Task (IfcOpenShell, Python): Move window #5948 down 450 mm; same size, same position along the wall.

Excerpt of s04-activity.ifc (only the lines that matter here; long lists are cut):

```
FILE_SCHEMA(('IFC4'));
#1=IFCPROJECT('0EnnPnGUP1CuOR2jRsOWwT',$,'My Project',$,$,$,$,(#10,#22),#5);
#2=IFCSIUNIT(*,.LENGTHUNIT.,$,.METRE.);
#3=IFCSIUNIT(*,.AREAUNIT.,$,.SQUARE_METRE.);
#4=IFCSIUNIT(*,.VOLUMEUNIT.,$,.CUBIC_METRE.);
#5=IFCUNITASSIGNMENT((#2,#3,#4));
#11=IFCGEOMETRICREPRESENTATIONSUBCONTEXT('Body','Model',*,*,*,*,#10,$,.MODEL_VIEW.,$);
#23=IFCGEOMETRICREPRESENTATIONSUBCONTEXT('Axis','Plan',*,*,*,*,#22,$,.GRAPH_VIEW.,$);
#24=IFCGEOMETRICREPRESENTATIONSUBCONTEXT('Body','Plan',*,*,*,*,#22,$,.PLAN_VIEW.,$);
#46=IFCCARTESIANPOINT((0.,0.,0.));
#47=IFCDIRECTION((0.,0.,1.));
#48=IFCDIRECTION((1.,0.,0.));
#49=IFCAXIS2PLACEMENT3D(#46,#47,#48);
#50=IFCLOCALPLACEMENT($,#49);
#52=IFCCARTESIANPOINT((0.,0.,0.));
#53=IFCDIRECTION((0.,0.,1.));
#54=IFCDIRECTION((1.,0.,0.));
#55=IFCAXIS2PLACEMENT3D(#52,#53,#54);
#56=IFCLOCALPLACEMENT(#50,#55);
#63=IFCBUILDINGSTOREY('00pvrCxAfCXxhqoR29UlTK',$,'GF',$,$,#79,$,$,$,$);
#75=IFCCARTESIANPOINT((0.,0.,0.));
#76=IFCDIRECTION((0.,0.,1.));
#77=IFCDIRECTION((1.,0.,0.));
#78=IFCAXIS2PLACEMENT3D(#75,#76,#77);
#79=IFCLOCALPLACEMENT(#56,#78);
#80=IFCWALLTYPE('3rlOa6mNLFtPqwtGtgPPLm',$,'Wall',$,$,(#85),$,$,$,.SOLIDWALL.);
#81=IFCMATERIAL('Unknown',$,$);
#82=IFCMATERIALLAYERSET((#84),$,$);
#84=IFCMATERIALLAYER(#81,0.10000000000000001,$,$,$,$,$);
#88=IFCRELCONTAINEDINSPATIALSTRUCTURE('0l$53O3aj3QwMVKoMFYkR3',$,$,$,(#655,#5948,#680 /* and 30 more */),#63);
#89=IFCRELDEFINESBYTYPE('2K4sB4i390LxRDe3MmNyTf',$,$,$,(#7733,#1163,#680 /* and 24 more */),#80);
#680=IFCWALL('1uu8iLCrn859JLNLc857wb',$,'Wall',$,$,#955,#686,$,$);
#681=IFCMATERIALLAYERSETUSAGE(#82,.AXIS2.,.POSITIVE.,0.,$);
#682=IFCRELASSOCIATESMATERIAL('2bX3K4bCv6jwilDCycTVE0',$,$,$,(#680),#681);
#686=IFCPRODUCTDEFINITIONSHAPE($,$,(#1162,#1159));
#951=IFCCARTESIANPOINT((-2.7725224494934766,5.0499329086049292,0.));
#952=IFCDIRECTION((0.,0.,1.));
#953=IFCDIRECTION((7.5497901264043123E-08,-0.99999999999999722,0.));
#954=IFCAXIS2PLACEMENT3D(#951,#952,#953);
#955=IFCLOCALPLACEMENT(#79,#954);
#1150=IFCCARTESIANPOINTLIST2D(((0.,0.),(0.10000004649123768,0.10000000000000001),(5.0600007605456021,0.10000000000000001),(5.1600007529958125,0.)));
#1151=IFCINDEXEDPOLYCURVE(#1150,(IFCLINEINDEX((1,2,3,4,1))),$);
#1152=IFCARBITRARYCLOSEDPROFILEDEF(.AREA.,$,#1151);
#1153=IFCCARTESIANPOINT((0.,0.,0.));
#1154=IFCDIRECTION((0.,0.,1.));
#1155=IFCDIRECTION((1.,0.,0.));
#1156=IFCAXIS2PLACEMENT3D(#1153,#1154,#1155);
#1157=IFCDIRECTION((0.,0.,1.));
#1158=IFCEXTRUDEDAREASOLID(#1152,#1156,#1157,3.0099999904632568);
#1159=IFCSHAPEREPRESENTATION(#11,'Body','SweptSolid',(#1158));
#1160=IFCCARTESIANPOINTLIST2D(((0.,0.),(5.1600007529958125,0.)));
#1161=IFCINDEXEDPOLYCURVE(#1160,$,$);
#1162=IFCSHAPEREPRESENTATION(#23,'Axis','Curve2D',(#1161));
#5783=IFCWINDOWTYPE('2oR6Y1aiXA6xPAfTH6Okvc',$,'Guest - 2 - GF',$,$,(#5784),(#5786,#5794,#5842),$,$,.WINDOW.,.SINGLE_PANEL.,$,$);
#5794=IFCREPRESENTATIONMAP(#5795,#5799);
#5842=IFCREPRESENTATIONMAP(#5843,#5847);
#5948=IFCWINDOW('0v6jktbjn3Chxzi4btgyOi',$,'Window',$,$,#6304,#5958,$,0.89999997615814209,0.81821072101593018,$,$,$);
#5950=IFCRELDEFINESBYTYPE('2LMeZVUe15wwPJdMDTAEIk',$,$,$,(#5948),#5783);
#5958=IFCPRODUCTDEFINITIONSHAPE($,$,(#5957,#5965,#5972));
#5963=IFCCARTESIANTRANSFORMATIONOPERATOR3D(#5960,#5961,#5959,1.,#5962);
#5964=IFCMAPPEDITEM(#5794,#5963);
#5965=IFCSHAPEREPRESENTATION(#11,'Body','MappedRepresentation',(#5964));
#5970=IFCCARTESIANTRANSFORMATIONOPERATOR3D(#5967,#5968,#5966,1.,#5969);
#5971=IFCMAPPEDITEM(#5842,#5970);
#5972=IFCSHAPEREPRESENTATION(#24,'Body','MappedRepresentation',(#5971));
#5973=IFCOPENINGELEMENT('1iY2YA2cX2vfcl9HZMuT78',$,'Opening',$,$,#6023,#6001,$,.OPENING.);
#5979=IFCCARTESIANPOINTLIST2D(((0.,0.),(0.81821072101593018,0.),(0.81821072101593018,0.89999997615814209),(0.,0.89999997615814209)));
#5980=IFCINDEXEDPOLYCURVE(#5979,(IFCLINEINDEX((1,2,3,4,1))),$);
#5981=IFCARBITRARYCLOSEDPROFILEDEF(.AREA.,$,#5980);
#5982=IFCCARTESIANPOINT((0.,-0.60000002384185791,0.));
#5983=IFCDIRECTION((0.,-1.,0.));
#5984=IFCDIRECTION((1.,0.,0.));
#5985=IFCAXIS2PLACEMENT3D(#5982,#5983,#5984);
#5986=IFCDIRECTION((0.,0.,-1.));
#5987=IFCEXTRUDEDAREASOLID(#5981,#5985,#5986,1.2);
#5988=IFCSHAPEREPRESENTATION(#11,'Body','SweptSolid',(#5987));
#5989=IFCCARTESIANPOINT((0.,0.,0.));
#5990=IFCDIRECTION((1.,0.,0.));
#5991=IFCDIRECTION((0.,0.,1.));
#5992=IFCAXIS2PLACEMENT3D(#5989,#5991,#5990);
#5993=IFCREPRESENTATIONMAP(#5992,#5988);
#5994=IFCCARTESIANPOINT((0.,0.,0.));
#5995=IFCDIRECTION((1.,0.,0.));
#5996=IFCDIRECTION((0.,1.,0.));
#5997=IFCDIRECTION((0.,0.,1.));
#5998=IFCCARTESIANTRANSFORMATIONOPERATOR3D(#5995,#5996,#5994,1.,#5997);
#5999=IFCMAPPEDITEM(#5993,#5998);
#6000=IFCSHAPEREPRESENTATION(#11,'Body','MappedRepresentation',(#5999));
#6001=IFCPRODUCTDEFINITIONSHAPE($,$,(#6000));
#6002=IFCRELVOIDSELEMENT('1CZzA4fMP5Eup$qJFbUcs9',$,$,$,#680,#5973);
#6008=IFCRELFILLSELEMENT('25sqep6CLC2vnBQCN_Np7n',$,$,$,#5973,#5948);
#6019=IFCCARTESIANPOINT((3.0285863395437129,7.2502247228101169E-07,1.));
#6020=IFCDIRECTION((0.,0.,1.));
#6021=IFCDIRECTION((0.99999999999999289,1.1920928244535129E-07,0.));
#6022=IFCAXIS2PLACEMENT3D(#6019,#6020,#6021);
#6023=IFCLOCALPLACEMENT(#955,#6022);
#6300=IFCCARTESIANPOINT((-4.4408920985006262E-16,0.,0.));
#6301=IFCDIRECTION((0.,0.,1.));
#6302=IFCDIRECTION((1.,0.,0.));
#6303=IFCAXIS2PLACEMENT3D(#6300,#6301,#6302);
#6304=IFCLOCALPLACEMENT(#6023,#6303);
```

```python
import numpy as np
import ifcopenshell
import ifcopenshell.api.geometry
import ifcopenshell.util.placement
import ifcopenshell.util.unit

model = ifcopenshell.open("s04-activity.ifc")
unit_scale = ifcopenshell.util.unit.calculate_unit_scale(model)

window = model.by_id(5948)
opening = window.FillsVoids[0].RelatingOpeningElement
dz = -0.45 / unit_scale

shift = np.array([0.0, 0.0, dz])
# The window is placed relative to its opening, so it follows when the opening moves.
matrix = ifcopenshell.util.placement.get_local_placement(opening.ObjectPlacement)
matrix[:3, 3] += shift
ifcopenshell.api.geometry.edit_object_placement(
    model, product=opening, matrix=matrix, is_si=False, should_transform_children=True
)

print(f"moved by {dz * unit_scale:+.3f} m")

model.write("s04-activity-out.ifc")
```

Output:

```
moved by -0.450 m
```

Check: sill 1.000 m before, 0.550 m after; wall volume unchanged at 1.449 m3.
